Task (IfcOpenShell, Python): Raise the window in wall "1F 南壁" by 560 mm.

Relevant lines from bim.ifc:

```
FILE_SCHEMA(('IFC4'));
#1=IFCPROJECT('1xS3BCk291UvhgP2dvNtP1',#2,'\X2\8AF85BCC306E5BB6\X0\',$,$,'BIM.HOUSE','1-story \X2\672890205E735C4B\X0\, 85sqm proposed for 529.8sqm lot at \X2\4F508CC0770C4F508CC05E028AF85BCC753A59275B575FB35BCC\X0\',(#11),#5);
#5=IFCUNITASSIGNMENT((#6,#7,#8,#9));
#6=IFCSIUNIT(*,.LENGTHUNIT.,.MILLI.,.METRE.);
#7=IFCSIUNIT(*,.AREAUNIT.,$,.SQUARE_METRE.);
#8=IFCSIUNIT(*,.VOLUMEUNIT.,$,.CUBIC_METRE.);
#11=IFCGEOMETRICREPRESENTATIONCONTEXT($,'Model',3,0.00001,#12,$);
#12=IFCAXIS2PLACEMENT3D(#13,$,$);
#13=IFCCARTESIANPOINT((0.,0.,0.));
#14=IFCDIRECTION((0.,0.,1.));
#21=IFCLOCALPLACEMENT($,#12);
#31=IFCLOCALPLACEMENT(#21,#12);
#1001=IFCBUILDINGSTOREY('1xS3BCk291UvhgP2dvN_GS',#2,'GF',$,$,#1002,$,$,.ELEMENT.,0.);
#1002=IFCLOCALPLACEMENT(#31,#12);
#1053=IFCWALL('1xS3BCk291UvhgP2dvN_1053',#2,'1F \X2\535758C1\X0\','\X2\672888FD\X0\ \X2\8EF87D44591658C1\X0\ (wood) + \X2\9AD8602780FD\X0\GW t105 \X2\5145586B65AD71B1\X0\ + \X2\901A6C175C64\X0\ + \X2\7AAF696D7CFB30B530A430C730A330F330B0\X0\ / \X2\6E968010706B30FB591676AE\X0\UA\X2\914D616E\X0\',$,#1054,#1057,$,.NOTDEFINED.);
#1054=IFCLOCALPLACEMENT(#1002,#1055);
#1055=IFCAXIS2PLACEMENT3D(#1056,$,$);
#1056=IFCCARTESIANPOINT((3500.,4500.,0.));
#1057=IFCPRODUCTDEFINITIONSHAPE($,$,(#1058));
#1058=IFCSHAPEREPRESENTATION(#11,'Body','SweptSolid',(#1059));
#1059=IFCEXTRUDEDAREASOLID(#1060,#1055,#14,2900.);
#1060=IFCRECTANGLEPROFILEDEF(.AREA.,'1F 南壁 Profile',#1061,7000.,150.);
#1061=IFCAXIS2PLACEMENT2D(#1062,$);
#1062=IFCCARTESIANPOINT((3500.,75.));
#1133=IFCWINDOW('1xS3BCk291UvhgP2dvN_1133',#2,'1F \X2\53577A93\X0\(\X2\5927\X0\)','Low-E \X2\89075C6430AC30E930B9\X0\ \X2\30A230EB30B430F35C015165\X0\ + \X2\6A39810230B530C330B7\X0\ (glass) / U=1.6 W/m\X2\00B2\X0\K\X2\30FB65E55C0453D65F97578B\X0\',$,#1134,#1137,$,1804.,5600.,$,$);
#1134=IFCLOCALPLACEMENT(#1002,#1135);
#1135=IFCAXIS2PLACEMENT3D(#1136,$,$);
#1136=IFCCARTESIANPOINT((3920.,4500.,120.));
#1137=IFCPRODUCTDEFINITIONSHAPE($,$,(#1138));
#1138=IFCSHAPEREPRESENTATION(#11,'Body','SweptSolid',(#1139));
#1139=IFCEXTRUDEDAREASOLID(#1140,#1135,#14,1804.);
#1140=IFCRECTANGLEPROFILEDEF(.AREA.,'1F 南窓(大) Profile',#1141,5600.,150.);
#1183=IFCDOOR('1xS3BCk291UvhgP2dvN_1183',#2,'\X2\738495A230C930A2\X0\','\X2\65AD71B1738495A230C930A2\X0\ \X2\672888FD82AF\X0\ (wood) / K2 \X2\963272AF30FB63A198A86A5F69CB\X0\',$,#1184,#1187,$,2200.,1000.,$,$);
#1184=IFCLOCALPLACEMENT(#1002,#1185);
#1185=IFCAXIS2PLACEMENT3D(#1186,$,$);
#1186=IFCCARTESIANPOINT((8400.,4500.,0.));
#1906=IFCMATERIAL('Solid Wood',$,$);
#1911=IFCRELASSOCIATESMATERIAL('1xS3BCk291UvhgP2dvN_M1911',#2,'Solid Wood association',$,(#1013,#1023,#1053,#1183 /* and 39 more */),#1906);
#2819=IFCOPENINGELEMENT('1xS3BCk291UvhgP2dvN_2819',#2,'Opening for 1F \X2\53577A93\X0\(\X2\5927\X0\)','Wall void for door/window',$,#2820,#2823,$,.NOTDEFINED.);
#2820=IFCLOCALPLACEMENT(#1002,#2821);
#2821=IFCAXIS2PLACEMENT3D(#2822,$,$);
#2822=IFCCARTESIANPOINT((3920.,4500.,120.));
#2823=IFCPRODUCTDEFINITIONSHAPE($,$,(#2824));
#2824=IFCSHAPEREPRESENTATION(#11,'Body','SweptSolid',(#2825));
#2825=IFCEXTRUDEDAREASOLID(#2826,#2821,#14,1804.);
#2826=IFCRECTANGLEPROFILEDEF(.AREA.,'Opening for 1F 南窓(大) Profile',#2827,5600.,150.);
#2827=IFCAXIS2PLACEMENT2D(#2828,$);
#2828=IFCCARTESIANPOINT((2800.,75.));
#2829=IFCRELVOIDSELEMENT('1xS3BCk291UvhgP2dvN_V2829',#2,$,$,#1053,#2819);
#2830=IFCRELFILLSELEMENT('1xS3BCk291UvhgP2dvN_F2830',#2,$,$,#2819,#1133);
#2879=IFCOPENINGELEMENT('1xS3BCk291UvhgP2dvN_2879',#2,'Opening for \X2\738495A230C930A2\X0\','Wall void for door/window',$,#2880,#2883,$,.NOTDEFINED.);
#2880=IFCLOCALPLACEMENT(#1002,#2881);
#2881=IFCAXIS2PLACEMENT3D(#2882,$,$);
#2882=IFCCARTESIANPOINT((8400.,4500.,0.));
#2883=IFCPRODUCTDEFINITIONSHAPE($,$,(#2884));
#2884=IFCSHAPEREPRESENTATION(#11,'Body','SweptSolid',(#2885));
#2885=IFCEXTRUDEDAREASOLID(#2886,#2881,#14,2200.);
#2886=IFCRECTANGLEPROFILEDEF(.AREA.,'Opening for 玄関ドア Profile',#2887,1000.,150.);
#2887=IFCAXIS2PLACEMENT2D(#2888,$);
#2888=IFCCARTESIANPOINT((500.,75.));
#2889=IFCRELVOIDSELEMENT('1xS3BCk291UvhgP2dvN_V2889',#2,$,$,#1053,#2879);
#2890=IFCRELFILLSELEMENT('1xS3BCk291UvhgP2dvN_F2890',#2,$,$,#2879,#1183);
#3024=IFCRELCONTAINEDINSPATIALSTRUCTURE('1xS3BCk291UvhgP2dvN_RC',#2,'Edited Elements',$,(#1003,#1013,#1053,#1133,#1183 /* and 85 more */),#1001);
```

```python
import numpy as np
import ifcopenshell
import ifcopenshell.api.geometry
import ifcopenshell.util.placement
import ifcopenshell.util.unit

model = ifcopenshell.open("bim.ifc")
unit_scale = ifcopenshell.util.unit.calculate_unit_scale(model)

window = model.by_guid("1xS3BCk291UvhgP2dvN_1133")
opening = window.FillsVoids[0].RelatingOpeningElement
dz = 0.56 / unit_scale

shift = np.array([0.0, 0.0, dz])
# The window is not placed relative to its opening, so move both.
for product in (opening, window):
    matrix = ifcopenshell.util.placement.get_local_placement(product.ObjectPlacement)
    matrix[:3, 3] += shift
    ifcopenshell.api.geometry.edit_object_placement(model, product=product, matrix=matrix, is_si=False)

print(f"moved by {dz * unit_scale:+.3f} m")

model.write("bim_rev.ifc")
```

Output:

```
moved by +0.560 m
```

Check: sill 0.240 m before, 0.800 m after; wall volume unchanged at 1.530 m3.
